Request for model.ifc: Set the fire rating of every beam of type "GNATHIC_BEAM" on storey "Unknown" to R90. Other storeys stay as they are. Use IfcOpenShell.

First a look at what the model holds.

```python
import ifcopenshell
import ifcopenshell.util.element

model = ifcopenshell.open("model.ifc")
print(model.schema)
storey = next(s for s in model.by_type("IfcBuildingStorey") if s.Name == "Unknown")
beams = [e for e in ifcopenshell.util.element.get_decomposition(storey) if e.is_a("IfcBeam")]
seen = {}
for e in beams:
    element_type = ifcopenshell.util.element.get_type(e)
    key = (element_type.Name if element_type != e and element_type else None, ifcopenshell.util.element.get_pset(e, "Pset_BeamCommon", "FireRating"))
    seen[key] = seen.get(key, 0) + 1
for (name, value), count in sorted(seen.items(), key=str):
    print(count, "x", name, "|", value)
```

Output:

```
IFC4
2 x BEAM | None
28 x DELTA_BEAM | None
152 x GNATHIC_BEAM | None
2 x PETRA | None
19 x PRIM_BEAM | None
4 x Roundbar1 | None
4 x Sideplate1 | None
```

```python
import ifcopenshell
import ifcopenshell.api.pset
import ifcopenshell.util.element

model = ifcopenshell.open("model.ifc")

storey = next(s for s in model.by_type("IfcBuildingStorey") if s.Name == "Unknown")
beams = [e for e in ifcopenshell.util.element.get_decomposition(storey) if e.is_a("IfcBeam")]

count = 0
for e in beams:
    element_type = ifcopenshell.util.element.get_type(e)
    if element_type in (None, e) or element_type.Name != "GNATHIC_BEAM":
        continue
    found = ifcopenshell.util.element.get_pset(e, "Pset_BeamCommon", should_inherit=False)
    if found:
        pset = model.by_id(found["id"])
        if len(ifcopenshell.util.element.get_elements_by_pset(pset)) > 1:
            pset = ifcopenshell.api.pset.unshare_pset(model, products=[e], pset=pset)[0]
    else:
        pset = ifcopenshell.api.pset.add_pset(model, product=e, name="Pset_BeamCommon")
    ifcopenshell.api.pset.edit_pset(model, pset=pset, properties={"FireRating": "R90"})
    count += 1

print(count, "beams updated")

model.write("model_v2.ifc")
```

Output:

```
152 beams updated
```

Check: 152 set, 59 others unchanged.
